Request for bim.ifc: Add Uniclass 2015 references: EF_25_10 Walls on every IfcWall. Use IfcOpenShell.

First a look at what the model holds.

```python
import ifcopenshell

model = ifcopenshell.open("bim.ifc")
print(model.schema)
print("classifications:", [c.Name for c in model.by_type("IfcClassification")])
for ifc_class in ("IfcDoor", "IfcRoof", "IfcStair", "IfcWall", "IfcWindow"):
    print(ifc_class, len(model.by_type(ifc_class)))
```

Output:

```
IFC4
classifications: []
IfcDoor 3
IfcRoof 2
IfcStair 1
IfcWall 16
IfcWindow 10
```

```python
import ifcopenshell
import ifcopenshell.api.classification

model = ifcopenshell.open("bim.ifc")

system = ifcopenshell.api.classification.add_classification(model, classification="Uniclass 2015")

codes = {
    "IfcWall": ("EF_25_10", "Walls"),
}
for ifc_class, (code, name) in codes.items():
    products = model.by_type(ifc_class)
    ifcopenshell.api.classification.add_reference(
        model, products=products, classification=system, identification=code, name=name
    )
    print(code, len(products))

model.write("bim-out.ifc")
```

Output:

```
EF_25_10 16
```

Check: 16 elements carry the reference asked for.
